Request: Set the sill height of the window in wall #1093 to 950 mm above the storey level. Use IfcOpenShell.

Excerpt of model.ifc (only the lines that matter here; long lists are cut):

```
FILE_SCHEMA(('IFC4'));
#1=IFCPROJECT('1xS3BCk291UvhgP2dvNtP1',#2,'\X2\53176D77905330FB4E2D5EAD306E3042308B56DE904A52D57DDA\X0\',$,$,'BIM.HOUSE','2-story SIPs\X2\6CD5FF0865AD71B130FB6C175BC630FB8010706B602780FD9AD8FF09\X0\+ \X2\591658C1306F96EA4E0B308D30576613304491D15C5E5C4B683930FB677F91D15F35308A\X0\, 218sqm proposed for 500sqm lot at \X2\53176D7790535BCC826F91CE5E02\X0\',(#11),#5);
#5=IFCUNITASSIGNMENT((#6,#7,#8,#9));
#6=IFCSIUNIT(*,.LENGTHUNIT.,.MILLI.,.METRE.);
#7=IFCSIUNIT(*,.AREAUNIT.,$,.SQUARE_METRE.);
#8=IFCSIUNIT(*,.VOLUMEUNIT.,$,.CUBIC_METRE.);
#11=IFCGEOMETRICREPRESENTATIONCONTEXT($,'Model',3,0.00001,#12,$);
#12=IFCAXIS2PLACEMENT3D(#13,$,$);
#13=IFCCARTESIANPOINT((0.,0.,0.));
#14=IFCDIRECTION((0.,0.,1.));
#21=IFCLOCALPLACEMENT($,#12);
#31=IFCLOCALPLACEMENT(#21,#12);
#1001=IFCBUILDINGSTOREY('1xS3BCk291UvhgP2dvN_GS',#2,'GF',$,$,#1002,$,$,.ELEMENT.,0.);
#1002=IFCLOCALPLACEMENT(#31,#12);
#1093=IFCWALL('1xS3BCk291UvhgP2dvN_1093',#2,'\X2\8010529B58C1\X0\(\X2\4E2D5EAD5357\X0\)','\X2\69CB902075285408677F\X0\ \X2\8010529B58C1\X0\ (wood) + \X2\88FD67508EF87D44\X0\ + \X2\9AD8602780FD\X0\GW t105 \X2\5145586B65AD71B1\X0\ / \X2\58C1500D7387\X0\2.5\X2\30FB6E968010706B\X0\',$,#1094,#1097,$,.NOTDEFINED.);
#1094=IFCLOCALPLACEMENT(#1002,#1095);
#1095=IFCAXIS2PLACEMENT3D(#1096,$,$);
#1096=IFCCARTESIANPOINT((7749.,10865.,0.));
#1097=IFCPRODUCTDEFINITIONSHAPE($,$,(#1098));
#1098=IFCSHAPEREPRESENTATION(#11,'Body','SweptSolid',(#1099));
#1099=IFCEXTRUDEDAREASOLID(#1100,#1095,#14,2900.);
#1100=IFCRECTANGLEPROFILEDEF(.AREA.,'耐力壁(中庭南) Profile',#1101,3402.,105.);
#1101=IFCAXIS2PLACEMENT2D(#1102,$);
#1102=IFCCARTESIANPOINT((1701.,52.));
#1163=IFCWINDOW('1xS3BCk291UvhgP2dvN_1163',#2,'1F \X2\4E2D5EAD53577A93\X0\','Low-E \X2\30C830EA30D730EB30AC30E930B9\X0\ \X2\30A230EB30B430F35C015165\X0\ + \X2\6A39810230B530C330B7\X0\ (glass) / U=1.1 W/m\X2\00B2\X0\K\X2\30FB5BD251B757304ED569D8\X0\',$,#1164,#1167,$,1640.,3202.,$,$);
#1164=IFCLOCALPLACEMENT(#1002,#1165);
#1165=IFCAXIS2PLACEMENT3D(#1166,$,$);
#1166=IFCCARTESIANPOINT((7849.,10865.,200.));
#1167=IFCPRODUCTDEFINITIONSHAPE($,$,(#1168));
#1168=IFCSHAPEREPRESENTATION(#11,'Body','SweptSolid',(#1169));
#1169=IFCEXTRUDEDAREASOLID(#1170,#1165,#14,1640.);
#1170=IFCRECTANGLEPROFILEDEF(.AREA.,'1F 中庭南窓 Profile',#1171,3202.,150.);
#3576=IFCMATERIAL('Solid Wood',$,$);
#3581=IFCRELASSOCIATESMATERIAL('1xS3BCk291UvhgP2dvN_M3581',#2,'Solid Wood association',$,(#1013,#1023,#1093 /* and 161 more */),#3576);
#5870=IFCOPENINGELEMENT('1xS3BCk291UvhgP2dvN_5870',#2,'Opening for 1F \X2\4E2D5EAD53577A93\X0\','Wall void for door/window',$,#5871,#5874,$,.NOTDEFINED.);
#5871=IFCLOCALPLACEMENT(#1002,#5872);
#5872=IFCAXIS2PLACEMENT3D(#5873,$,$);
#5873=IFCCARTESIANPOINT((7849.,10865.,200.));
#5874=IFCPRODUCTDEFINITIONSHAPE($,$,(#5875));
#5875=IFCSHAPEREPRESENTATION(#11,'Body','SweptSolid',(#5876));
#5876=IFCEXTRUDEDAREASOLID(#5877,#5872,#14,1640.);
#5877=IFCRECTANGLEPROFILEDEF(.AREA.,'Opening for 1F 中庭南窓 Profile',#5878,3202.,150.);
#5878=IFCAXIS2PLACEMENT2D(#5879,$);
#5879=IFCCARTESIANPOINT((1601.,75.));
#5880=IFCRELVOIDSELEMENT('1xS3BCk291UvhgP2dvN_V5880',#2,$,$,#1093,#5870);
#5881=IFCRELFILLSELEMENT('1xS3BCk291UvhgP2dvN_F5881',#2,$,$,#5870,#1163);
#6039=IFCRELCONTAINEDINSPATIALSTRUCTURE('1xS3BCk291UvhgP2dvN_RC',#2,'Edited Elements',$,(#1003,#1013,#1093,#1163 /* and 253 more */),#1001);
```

```python
import numpy as np
import ifcopenshell
import ifcopenshell.api.geometry
import ifcopenshell.geom
import ifcopenshell.util.element
import ifcopenshell.util.placement
import ifcopenshell.util.shape
import ifcopenshell.util.unit

model = ifcopenshell.open("model.ifc")
unit_scale = ifcopenshell.util.unit.calculate_unit_scale(model)

window = model.by_guid("1xS3BCk291UvhgP2dvN_1163")
opening = window.FillsVoids[0].RelatingOpeningElement
storey = ifcopenshell.util.element.get_container(window, ifc_class="IfcBuildingStorey")
level = ifcopenshell.util.placement.get_local_placement(storey.ObjectPlacement)[2, 3]

# The opening's origin need not be at the sill, so measure its lowest point.
shape = ifcopenshell.geom.create_shape(ifcopenshell.geom.settings(), opening)
bottom = ifcopenshell.util.shape.get_shape_bottom_elevation(shape, shape.geometry) / unit_scale
dz = level + 950.0 - bottom

shift = np.array([0.0, 0.0, dz])
# The window is not placed relative to its opening, so move both.
for product in (opening, window):
    matrix = ifcopenshell.util.placement.get_local_placement(product.ObjectPlacement)
    matrix[:3, 3] += shift
    ifcopenshell.api.geometry.edit_object_placement(model, product=product, matrix=matrix, is_si=False)

print(f"moved by {dz * unit_scale:+.3f} m")

model.write("model_v2.ifc")
```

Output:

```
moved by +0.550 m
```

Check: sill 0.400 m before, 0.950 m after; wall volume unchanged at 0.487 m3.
